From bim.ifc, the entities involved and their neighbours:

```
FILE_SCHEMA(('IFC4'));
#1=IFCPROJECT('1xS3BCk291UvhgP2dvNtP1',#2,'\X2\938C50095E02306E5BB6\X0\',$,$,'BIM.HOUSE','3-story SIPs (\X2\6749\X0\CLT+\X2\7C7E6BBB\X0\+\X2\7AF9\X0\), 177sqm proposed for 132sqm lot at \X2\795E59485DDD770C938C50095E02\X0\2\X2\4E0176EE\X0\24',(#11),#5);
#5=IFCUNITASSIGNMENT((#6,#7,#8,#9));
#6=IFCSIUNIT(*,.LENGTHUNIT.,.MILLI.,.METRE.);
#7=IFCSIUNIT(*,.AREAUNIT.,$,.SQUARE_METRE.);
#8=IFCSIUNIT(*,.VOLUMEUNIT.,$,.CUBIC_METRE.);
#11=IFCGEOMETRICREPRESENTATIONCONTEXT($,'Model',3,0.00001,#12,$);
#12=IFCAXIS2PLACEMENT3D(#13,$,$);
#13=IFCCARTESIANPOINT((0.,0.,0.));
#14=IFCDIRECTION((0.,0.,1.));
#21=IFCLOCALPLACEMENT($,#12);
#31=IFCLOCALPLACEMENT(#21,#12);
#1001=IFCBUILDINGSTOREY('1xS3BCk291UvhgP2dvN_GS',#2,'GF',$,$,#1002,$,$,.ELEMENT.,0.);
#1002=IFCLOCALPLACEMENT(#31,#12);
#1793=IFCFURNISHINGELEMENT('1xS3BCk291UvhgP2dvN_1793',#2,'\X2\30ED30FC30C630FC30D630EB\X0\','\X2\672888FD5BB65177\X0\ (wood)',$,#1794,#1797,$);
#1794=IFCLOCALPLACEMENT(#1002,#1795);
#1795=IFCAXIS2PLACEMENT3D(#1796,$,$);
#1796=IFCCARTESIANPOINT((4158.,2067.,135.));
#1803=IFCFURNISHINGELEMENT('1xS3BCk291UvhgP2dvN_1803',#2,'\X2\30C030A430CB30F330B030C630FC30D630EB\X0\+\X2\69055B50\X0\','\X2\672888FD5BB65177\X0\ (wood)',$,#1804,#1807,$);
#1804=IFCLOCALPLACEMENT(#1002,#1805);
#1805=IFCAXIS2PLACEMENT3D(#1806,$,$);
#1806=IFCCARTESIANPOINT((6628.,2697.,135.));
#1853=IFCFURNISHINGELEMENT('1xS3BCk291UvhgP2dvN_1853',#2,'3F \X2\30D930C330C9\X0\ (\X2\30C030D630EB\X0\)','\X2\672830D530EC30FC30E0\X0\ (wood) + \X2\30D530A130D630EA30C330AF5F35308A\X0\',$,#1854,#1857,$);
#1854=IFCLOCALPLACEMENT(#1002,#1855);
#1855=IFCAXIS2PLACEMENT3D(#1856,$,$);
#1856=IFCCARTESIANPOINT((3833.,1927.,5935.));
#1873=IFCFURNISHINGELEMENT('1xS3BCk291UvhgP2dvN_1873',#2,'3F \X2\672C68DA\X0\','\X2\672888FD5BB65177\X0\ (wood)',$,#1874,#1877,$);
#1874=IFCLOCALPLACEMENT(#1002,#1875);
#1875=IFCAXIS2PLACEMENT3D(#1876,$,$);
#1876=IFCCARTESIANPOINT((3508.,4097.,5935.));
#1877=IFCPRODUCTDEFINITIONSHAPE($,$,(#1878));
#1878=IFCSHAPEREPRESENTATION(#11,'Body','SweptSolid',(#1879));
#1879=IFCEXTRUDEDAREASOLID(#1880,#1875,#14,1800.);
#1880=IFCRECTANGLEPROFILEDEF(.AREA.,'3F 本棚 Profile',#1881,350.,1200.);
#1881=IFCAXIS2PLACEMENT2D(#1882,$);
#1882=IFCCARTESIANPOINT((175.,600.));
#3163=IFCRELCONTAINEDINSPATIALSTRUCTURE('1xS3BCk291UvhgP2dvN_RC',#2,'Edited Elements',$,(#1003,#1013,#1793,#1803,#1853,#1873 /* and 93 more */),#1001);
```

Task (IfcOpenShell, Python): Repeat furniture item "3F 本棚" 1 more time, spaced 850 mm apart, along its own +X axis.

```python
import ifcopenshell
import ifcopenshell.api.geometry
import ifcopenshell.api.root
import ifcopenshell.util.element
import ifcopenshell.util.placement
import ifcopenshell.util.unit

model = ifcopenshell.open("bim.ifc")
unit_scale = ifcopenshell.util.unit.calculate_unit_scale(model)


def reuse_history(source, copy):
    """copy_class also copies each property set's owner history, people and application; keep the originals."""
    for rel in copy.IsDefinedBy:
        if rel.is_a("IfcRelDefinesByProperties") and (history := rel.RelatingPropertyDefinition.OwnerHistory):
            rel.RelatingPropertyDefinition.OwnerHistory = source.OwnerHistory
            ifcopenshell.util.element.remove_deep2(model, history)


source = model.by_guid("1xS3BCk291UvhgP2dvN_1873")
base = ifcopenshell.util.placement.get_local_placement(source.ObjectPlacement)
step = base[:3, 0] * 0.85 / unit_scale

for i in range(1, 2):
    copy = ifcopenshell.api.root.copy_class(model, product=source)
    copy.Representation = ifcopenshell.util.element.copy_deep(
        model, source.Representation, exclude=["IfcGeometricRepresentationContext", "IfcRepresentationMap"]
    )
    reuse_history(source, copy)
    matrix = base.copy()
    matrix[:3, 3] += i * step
    print("added at", matrix[:3, 3].round(3) + 0.0)
    ifcopenshell.api.geometry.edit_object_placement(model, product=copy, matrix=matrix, is_si=False)

model.write("bim_rev.ifc")
```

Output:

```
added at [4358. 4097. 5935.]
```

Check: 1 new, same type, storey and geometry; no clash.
